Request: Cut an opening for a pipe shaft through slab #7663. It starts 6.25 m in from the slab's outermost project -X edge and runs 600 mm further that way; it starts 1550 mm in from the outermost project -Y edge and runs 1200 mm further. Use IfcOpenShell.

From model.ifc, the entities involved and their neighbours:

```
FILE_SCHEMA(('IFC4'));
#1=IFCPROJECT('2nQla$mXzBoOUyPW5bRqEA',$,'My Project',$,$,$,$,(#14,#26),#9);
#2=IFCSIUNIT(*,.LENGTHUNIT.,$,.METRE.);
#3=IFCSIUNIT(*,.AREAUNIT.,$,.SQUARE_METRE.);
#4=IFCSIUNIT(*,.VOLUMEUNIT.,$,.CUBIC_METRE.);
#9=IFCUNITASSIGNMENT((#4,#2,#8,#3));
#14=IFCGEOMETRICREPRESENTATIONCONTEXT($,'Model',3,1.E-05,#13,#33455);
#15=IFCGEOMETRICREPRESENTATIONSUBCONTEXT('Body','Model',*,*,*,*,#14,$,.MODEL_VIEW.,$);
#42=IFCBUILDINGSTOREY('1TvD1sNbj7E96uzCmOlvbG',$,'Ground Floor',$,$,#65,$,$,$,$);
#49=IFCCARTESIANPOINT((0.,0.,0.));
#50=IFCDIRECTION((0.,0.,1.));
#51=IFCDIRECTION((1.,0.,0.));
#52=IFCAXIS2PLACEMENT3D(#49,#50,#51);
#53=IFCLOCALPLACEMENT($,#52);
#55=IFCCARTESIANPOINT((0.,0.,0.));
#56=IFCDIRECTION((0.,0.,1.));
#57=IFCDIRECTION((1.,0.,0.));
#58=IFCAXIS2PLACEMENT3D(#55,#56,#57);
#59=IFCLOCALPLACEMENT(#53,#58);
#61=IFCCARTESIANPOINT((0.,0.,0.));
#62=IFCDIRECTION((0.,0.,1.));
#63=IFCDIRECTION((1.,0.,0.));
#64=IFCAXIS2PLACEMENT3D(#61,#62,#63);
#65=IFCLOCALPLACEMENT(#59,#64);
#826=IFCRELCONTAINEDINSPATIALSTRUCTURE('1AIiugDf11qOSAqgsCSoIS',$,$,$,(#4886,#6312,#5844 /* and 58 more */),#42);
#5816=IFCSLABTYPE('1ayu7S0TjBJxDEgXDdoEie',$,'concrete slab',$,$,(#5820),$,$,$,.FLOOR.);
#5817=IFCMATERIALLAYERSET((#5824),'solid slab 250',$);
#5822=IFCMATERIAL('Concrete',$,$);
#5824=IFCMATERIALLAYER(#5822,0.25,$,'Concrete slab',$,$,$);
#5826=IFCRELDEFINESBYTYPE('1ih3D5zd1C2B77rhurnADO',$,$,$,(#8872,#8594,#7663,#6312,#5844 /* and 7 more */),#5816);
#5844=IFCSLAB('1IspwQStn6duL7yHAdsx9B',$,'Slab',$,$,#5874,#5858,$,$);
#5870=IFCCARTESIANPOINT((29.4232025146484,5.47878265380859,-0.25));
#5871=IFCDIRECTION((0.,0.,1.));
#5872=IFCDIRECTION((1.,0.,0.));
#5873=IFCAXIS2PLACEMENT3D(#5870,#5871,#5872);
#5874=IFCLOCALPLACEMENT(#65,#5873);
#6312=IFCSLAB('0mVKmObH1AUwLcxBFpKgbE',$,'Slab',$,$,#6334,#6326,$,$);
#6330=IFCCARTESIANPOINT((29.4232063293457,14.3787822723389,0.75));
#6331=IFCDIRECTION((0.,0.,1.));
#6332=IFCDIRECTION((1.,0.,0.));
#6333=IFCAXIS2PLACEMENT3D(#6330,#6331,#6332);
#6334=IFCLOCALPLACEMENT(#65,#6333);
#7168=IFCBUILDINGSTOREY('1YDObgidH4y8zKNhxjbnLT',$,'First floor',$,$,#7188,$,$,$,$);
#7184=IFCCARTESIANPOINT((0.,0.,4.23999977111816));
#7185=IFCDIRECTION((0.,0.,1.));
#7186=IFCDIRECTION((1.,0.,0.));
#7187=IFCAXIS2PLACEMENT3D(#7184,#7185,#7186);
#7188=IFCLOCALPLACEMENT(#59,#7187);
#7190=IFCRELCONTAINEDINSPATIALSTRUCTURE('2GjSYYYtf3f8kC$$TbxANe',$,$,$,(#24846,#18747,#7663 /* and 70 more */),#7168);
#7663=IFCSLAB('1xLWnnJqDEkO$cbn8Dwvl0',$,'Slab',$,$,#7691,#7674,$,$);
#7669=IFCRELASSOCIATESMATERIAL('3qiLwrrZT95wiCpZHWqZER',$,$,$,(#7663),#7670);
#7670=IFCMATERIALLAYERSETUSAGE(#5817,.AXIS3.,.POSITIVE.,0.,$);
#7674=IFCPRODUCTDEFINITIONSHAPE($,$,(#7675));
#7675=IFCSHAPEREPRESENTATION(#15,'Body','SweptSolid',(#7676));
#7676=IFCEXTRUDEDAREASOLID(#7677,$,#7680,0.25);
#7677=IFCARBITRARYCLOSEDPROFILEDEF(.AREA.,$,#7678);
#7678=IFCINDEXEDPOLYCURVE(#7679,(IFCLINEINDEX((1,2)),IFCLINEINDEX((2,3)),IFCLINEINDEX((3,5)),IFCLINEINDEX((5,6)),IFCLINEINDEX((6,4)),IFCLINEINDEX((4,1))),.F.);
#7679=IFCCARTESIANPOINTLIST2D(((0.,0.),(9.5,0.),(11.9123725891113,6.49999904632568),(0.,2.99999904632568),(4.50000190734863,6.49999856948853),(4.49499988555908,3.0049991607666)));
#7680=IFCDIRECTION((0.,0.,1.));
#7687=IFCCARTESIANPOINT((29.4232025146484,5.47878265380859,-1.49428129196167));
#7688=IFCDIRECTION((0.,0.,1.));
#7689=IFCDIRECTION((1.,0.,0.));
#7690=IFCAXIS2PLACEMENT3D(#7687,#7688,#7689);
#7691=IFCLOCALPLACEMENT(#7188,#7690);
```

```python
import numpy as np
import ifcopenshell
import ifcopenshell.api.feature
import ifcopenshell.api.geometry
import ifcopenshell.api.root
import ifcopenshell.geom
import ifcopenshell.util.placement
import ifcopenshell.util.representation
import ifcopenshell.util.shape
import ifcopenshell.util.unit

model = ifcopenshell.open("model.ifc")
unit_scale = ifcopenshell.util.unit.calculate_unit_scale(model)
settings = ifcopenshell.geom.settings()


def volume(element):
    """Net volume in cubic metres, openings subtracted."""
    shape = ifcopenshell.geom.create_shape(settings, element)
    return ifcopenshell.util.shape.get_volume(shape.geometry)


slab = model.by_id(7663)
before = volume(slab)

# Extent in the slab's own axes, in metres. The edges named are its -X and -Y sides.
slab_shape = ifcopenshell.geom.create_shape(settings, slab)
vertices = ifcopenshell.util.shape.get_vertices(slab_shape.geometry)
x_min, y_min, bottom = vertices.min(axis=0)
top = vertices[:, 2].max()

opening = ifcopenshell.api.root.create_entity(model, ifc_class="IfcOpeningElement", name="Pipe shaft opening", predefined_type="OPENING")
context = ifcopenshell.util.representation.get_context(model, "Model", "Body", "MODEL_VIEW")
width, depth = 0.6, 1.2
outline = [(0.0, 0.0), (width, 0.0), (width, depth), (0.0, depth), (0.0, 0.0)]
# Overshoot both faces by 50 mm so the cut is clean.
shape = ifcopenshell.api.geometry.add_slab_representation(
    model, context=context, depth=top - bottom + 0.1, polyline=outline
)
ifcopenshell.api.geometry.assign_representation(model, product=opening, representation=shape)

matrix = ifcopenshell.util.placement.get_local_placement(slab.ObjectPlacement)
matrix[:, 3] = matrix @ np.append(np.array([x_min + 6.25, y_min + 1.55, bottom - 0.05]) / unit_scale, 1.0)
ifcopenshell.api.geometry.edit_object_placement(model, product=opening, matrix=matrix, is_si=False)
ifcopenshell.api.feature.add_feature(model, feature=opening, element=slab)

after = volume(slab)

print(f"slab volume {before:.3f} -> {after:.3f} m3")

model.write("model_edited.ifc")
```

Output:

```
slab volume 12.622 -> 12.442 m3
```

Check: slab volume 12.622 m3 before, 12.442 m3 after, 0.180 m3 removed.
